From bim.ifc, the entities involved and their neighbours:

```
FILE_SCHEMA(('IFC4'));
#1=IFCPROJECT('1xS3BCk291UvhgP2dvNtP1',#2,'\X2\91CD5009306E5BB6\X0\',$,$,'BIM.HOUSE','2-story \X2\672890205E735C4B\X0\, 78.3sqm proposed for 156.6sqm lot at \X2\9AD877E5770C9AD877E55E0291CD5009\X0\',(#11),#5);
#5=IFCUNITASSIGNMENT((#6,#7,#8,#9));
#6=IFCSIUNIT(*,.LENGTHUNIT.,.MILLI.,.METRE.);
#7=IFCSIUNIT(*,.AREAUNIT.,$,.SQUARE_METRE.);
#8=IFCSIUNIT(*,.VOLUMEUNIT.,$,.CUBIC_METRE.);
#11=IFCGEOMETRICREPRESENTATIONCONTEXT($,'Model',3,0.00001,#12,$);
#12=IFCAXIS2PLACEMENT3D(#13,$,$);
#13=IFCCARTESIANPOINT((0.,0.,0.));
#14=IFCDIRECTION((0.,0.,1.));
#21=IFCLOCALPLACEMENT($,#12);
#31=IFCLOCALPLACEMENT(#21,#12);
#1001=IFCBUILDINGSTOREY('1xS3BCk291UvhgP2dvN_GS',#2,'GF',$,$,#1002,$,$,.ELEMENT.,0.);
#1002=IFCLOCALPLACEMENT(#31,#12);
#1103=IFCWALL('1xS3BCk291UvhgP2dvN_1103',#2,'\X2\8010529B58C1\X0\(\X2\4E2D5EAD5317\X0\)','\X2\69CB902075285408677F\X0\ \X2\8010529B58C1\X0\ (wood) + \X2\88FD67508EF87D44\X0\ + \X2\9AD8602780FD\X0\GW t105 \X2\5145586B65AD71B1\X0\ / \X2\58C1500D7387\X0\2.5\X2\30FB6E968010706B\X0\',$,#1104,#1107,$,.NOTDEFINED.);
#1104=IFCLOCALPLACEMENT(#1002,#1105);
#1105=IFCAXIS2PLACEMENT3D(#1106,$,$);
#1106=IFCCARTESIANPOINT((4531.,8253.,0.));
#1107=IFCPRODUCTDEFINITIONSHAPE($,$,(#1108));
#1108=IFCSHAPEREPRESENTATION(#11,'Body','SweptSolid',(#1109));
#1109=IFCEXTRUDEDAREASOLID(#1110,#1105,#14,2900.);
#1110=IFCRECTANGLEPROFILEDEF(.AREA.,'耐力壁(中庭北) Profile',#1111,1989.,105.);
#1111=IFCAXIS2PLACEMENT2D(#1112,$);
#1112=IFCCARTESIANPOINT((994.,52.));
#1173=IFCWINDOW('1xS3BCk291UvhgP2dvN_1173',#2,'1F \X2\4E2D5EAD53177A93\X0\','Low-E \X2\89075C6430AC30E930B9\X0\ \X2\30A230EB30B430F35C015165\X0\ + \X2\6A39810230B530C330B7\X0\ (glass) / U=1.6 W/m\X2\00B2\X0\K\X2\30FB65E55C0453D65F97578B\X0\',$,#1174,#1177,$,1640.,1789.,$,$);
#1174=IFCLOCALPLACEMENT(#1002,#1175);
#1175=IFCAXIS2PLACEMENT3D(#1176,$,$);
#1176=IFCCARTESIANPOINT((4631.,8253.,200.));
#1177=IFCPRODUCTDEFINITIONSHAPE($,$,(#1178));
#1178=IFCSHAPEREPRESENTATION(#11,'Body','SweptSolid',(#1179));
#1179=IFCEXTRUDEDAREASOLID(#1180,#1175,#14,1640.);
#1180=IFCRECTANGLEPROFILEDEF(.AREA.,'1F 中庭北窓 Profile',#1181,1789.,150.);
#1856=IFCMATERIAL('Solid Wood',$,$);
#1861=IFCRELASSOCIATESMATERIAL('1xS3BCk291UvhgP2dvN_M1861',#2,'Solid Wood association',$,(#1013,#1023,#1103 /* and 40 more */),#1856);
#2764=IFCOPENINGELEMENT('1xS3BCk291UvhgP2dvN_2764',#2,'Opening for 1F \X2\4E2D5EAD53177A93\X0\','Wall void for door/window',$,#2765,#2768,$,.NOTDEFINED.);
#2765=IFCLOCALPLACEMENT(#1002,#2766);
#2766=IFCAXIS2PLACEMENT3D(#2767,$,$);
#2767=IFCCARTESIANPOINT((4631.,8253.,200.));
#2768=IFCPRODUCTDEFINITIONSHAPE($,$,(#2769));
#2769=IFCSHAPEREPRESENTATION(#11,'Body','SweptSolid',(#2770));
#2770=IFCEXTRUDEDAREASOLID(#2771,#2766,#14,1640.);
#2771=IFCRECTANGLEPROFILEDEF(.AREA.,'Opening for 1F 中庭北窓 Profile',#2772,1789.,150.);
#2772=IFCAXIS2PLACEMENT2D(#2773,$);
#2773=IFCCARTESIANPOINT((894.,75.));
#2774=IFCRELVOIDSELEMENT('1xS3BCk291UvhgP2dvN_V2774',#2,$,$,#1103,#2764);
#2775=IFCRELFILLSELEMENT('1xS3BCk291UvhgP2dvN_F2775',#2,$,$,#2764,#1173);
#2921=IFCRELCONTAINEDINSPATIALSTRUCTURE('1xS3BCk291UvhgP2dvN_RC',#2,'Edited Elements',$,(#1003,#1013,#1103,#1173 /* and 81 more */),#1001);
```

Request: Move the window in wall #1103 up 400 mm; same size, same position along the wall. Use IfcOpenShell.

```python
import numpy as np
import ifcopenshell
import ifcopenshell.api.geometry
import ifcopenshell.util.placement
import ifcopenshell.util.unit

model = ifcopenshell.open("bim.ifc")
unit_scale = ifcopenshell.util.unit.calculate_unit_scale(model)

window = model.by_guid("1xS3BCk291UvhgP2dvN_1173")
opening = window.FillsVoids[0].RelatingOpeningElement
dz = 400.0

shift = np.array([0.0, 0.0, dz])
# The window is not placed relative to its opening, so move both.
for product in (opening, window):
    matrix = ifcopenshell.util.placement.get_local_placement(product.ObjectPlacement)
    matrix[:3, 3] += shift
    ifcopenshell.api.geometry.edit_object_placement(model, product=product, matrix=matrix, is_si=False)

print(f"moved by {dz * unit_scale:+.3f} m")

model.write("bim-out.ifc")
```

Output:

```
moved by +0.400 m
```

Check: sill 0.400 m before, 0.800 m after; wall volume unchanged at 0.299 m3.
